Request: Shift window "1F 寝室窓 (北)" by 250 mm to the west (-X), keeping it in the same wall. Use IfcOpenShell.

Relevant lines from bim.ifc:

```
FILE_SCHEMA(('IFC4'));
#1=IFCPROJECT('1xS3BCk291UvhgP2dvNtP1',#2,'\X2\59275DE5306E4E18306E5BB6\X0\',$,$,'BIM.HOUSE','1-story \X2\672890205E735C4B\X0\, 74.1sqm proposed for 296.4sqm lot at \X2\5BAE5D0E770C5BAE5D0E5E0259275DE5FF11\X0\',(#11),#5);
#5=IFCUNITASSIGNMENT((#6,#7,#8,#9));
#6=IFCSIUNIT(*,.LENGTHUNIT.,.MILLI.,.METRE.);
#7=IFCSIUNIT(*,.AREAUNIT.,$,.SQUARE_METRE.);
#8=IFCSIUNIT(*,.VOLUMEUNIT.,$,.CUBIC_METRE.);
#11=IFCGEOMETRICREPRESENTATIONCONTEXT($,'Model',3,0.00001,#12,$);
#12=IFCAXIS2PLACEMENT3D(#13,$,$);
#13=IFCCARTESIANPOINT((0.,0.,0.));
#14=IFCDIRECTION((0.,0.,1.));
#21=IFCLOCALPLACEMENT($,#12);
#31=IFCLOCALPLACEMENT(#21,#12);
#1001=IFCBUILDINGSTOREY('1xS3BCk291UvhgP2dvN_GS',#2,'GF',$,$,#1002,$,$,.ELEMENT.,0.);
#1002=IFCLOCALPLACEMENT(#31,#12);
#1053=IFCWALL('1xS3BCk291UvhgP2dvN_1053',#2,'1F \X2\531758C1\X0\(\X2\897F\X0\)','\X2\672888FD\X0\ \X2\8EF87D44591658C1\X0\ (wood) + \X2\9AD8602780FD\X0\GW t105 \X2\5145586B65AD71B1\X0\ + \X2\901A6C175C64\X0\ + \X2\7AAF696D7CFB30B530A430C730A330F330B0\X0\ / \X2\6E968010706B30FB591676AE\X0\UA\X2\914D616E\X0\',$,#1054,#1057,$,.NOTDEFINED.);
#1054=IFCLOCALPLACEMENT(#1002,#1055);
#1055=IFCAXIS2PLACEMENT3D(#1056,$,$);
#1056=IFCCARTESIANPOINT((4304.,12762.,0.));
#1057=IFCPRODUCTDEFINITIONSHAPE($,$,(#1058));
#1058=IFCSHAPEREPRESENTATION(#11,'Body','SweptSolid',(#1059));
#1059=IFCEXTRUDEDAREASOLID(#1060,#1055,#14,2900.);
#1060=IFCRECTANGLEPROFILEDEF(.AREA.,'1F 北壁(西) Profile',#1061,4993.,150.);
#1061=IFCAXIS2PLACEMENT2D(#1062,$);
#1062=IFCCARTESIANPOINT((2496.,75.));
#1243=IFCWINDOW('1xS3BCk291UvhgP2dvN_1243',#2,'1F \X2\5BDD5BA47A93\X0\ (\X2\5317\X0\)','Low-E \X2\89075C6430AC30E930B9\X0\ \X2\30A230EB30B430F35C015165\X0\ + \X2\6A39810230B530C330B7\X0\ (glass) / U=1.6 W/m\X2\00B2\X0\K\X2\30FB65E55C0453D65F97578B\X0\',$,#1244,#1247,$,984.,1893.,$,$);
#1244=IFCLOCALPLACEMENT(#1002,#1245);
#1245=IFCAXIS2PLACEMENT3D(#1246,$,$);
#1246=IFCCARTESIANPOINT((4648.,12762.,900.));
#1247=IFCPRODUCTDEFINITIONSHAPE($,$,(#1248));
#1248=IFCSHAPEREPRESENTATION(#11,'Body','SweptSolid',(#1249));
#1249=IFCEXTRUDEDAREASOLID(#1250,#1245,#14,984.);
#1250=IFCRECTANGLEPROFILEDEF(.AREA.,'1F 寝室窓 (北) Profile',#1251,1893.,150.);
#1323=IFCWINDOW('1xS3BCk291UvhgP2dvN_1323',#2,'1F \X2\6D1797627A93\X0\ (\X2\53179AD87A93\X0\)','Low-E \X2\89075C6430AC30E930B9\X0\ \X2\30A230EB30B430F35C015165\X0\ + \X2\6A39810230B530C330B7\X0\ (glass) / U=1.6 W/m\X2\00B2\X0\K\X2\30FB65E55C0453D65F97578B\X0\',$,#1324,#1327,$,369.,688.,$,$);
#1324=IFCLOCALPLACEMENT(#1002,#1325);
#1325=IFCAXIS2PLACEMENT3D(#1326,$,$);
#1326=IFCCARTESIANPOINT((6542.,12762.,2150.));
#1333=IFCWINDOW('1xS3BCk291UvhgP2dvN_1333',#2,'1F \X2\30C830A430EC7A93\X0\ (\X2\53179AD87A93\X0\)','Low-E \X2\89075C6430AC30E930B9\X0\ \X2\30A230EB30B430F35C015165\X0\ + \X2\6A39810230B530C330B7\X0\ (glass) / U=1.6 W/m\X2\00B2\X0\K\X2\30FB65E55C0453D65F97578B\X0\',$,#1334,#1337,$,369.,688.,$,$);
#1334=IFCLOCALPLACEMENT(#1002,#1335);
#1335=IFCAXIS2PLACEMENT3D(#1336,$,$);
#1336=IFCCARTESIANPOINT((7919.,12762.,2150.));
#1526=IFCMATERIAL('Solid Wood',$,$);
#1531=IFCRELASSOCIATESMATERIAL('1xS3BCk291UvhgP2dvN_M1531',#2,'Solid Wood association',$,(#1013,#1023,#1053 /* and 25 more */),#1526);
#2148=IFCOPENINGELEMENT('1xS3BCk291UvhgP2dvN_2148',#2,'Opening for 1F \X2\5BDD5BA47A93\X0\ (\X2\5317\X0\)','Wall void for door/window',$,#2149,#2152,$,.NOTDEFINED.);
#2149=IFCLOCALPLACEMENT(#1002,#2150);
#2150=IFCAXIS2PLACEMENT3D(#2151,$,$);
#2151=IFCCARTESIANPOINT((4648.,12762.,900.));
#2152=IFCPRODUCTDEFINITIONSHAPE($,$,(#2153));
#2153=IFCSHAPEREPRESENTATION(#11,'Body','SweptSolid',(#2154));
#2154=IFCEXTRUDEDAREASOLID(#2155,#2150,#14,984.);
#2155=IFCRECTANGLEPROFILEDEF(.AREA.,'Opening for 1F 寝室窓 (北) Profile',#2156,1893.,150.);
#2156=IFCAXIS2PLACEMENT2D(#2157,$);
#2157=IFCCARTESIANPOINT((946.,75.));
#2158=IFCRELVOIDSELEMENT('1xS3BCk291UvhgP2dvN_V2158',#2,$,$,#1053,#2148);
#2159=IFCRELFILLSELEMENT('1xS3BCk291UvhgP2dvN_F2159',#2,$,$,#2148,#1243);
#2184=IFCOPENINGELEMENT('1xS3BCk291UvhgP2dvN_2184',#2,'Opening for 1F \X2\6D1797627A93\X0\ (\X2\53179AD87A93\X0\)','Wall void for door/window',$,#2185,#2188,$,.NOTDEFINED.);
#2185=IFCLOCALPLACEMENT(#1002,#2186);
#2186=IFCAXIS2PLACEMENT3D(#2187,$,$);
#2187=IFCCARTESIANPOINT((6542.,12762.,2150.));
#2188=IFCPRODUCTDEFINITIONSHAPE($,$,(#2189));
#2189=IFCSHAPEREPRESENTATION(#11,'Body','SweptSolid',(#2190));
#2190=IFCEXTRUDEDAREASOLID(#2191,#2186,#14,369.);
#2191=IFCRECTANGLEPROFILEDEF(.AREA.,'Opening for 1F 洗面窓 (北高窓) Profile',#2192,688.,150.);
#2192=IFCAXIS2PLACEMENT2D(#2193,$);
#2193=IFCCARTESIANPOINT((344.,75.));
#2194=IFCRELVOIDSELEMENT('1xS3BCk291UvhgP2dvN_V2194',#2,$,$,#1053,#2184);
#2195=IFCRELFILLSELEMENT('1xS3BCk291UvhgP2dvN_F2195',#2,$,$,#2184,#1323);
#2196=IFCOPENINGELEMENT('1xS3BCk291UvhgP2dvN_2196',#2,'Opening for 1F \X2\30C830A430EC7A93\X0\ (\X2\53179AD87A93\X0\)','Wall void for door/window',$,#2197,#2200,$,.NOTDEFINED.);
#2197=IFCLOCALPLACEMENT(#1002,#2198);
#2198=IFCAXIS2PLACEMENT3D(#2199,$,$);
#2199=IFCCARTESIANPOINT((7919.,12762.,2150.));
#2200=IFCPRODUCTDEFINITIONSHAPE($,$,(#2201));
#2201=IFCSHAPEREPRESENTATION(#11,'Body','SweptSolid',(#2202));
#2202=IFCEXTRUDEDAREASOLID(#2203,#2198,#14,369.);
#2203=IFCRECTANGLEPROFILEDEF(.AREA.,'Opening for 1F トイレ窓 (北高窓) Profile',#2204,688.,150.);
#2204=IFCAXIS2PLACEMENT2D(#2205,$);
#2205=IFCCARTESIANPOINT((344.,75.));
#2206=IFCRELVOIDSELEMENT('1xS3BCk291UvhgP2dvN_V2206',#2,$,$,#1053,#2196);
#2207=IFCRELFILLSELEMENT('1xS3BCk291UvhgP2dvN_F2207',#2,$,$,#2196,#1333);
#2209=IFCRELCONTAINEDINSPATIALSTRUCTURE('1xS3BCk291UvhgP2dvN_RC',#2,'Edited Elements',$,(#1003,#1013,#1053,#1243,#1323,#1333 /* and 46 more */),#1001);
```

```python
import ifcopenshell
import ifcopenshell.api.geometry
import ifcopenshell.util.placement
import ifcopenshell.util.unit

model = ifcopenshell.open("bim.ifc")
unit_scale = ifcopenshell.util.unit.calculate_unit_scale(model)

window = model.by_id(1243)
opening = window.FillsVoids[0].RelatingOpeningElement
wall = opening.VoidsElements[0].RelatingBuildingElement

wall_matrix = ifcopenshell.util.placement.get_local_placement(wall.ObjectPlacement)
shift = wall_matrix[:3, 0] * -0.25 / unit_scale
before = ifcopenshell.util.placement.get_local_placement(window.ObjectPlacement)[:3, 3].copy()

# The window is not placed relative to its opening, so move both.
for product in (opening, window):
    matrix = ifcopenshell.util.placement.get_local_placement(product.ObjectPlacement)
    matrix[:3, 3] += shift
    ifcopenshell.api.geometry.edit_object_placement(model, product=product, matrix=matrix, is_si=False)

after = ifcopenshell.util.placement.get_local_placement(window.ObjectPlacement)[:3, 3]
print("window moved by", (after - before).round(3) + 0.0)

model.write("bim_v2.ifc")
```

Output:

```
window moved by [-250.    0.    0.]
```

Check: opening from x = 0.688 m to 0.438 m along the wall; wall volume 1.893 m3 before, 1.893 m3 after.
